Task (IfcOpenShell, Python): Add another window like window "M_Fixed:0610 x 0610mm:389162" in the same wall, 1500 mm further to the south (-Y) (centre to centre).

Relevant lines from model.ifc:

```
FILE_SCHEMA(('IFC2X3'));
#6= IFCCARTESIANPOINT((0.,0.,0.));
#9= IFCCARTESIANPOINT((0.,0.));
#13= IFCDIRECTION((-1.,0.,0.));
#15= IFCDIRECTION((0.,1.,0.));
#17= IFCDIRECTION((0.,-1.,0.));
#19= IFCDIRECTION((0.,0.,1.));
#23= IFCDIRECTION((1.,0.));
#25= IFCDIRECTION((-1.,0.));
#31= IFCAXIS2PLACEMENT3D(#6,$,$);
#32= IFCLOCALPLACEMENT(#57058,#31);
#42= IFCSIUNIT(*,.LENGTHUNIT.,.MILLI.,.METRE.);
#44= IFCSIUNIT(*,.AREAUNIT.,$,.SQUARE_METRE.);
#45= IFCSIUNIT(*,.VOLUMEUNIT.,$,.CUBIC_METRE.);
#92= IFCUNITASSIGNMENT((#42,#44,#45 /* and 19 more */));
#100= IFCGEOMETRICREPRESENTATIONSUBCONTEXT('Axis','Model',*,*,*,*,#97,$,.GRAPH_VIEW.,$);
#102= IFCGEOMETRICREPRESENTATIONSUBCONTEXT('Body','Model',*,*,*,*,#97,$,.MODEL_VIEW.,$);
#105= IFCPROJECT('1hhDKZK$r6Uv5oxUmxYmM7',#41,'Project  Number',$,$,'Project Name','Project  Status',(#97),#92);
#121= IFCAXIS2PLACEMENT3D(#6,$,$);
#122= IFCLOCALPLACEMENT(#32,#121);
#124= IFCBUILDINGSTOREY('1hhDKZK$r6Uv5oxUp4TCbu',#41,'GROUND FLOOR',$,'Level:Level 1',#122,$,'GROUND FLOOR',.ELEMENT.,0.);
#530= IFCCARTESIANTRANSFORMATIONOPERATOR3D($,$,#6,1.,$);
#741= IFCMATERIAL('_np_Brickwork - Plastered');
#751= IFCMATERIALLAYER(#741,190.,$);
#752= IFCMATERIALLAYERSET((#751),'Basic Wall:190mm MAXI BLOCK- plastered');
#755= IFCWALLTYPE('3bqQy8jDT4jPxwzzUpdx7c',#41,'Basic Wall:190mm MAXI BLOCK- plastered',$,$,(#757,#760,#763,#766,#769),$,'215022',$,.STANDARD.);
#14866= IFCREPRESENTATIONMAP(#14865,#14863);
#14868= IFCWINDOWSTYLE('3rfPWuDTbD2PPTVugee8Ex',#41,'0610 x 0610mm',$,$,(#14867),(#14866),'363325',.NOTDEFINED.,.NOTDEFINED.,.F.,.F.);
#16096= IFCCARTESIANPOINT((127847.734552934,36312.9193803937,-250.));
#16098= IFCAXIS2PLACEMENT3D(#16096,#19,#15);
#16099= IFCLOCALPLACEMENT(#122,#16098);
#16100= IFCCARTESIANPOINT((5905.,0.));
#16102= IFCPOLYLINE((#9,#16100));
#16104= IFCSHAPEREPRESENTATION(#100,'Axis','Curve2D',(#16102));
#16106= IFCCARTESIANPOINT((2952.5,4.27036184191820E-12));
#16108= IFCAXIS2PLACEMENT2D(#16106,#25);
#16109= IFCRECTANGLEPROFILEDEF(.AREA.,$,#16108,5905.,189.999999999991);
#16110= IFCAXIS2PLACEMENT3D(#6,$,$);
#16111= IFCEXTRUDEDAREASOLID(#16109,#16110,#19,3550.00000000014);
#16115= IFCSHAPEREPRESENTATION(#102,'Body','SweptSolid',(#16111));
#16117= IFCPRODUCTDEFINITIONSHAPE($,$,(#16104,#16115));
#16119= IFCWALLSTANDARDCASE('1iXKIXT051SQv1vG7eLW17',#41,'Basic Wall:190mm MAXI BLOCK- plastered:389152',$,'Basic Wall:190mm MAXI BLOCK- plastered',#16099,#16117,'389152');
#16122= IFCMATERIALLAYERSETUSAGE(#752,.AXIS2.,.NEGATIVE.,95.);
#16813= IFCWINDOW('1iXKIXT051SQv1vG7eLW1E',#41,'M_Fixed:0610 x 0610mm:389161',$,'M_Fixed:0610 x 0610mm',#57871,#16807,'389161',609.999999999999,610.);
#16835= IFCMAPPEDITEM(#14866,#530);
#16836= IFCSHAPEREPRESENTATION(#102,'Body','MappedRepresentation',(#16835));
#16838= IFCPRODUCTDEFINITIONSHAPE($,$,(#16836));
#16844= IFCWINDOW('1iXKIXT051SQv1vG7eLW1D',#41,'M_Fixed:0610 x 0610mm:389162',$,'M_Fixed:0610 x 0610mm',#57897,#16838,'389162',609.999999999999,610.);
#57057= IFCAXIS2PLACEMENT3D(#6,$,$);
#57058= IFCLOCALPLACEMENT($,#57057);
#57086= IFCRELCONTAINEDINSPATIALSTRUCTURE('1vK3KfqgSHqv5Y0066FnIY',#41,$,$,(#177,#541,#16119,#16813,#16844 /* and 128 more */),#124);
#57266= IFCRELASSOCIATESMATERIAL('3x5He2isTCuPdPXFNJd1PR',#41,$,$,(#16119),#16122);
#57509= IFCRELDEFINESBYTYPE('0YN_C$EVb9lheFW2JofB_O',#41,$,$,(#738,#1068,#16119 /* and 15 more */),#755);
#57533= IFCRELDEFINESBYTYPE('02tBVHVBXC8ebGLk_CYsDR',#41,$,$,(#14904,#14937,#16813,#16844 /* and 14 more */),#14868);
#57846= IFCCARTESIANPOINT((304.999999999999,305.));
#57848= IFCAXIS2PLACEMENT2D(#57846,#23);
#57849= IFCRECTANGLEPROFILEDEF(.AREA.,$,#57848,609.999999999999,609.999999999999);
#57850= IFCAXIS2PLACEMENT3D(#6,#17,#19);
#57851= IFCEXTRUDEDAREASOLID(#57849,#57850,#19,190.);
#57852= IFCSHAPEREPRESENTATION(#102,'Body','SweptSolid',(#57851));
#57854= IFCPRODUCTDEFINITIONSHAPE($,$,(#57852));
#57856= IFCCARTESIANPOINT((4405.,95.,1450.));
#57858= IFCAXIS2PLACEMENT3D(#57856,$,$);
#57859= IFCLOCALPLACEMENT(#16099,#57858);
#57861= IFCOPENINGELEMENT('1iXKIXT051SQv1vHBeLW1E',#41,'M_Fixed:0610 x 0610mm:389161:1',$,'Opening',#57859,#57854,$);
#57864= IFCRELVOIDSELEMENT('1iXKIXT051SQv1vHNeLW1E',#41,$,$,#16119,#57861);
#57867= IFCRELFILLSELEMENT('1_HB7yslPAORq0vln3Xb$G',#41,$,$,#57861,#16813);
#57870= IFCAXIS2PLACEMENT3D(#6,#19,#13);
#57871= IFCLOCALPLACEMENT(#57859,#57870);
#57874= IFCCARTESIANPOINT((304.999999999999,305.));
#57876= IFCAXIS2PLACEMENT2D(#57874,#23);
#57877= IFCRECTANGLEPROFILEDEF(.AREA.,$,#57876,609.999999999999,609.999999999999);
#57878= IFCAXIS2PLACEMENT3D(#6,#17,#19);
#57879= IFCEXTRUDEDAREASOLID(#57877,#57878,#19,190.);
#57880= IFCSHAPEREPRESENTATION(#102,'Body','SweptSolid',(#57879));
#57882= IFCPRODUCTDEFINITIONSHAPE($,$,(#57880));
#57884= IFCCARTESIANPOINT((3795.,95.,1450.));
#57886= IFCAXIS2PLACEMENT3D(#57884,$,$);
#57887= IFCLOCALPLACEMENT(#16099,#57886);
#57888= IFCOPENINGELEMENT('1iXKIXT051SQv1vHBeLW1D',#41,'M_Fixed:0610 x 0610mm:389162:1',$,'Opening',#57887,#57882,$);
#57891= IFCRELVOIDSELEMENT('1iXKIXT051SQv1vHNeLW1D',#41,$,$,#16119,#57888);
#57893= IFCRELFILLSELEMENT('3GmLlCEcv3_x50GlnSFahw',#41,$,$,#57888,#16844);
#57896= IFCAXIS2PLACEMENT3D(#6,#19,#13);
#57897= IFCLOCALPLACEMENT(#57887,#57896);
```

```python
import ifcopenshell
import ifcopenshell.api.feature
import ifcopenshell.api.geometry
import ifcopenshell.api.root
import ifcopenshell.geom
import ifcopenshell.util.element
import ifcopenshell.util.placement
import ifcopenshell.util.shape

model = ifcopenshell.open("model.ifc")
settings = ifcopenshell.geom.settings()


def volume(element):
    """Net volume in cubic metres, openings subtracted."""
    shape = ifcopenshell.geom.create_shape(settings, element)
    return ifcopenshell.util.shape.get_volume(shape.geometry)


def reuse_history(source, copy):
    """copy_class also copies each property set's owner history, people and application; keep the originals."""
    for rel in copy.IsDefinedBy:
        if rel.is_a("IfcRelDefinesByProperties") and (history := rel.RelatingPropertyDefinition.OwnerHistory):
            rel.RelatingPropertyDefinition.OwnerHistory = source.OwnerHistory
            ifcopenshell.util.element.remove_deep2(model, history)


window = model.by_id(16844)
opening = window.FillsVoids[0].RelatingOpeningElement
wall = opening.VoidsElements[0].RelatingBuildingElement
before = volume(wall)
shift = ifcopenshell.util.placement.get_local_placement(wall.ObjectPlacement)[:3, 0] * -1500.0

# copy_class copies the void relationship, type, container and properties, but no geometry.
new_opening = ifcopenshell.api.root.copy_class(model, product=opening)
new_opening.Representation = ifcopenshell.util.element.copy_deep(
    model, opening.Representation, exclude=["IfcGeometricRepresentationContext", "IfcRepresentationMap"]
)
new_opening.Name = "M_Fixed:0610 x 0610mm"
new_window = ifcopenshell.api.root.copy_class(model, product=window)
new_window.Representation = ifcopenshell.util.element.copy_deep(
    model, window.Representation, exclude=["IfcGeometricRepresentationContext", "IfcRepresentationMap"]
)
new_window.Name = "M_Fixed:0610 x 0610mm"
new_window.Tag = None
reuse_history(window, new_window)
fills = ifcopenshell.api.feature.add_filling(model, opening=new_opening, element=new_window)
fills.OwnerHistory = new_window.OwnerHistory  # required in IFC2X3

for old, new in ((opening, new_opening), (window, new_window)):
    matrix = ifcopenshell.util.placement.get_local_placement(old.ObjectPlacement)
    matrix[:3, 3] += shift
    ifcopenshell.api.geometry.edit_object_placement(model, product=new, matrix=matrix, is_si=False)

after = volume(wall)

print(f"wall volume {before:.3f} -> {after:.3f} m3")

model.write("model-out.ifc")
```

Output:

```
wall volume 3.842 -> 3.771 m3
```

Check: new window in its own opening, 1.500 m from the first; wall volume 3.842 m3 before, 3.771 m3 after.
